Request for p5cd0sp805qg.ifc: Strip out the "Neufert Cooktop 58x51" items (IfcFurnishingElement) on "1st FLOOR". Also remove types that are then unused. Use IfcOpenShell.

First a look at what the model holds.

```python
import ifcopenshell
import ifcopenshell.util.element

model = ifcopenshell.open("p5cd0sp805qg.ifc")
print(model.schema)
storey = next(s for s in model.by_type("IfcBuildingStorey") if s.Name == "1st FLOOR")
furniture = [e for e in ifcopenshell.util.element.get_decomposition(storey) if e.is_a("IfcFurnishingElement")]
seen = {}
for e in furniture:
    element_type = ifcopenshell.util.element.get_type(e)
    name = element_type.Name if element_type not in (None, e) else None
    seen[name] = seen.get(name, 0) + 1
for name, count in sorted(seen.items(), key=str):
    print(count, "x", name)
```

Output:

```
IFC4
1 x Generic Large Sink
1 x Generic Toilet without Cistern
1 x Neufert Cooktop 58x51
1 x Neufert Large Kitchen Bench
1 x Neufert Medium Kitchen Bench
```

```python
import ifcopenshell
import ifcopenshell.api.root
import ifcopenshell.util.element

model = ifcopenshell.open("p5cd0sp805qg.ifc")

storey = next(s for s in model.by_type("IfcBuildingStorey") if s.Name == "1st FLOOR")
furniture = [e for e in ifcopenshell.util.element.get_decomposition(storey) if e.is_a("IfcFurnishingElement")]
targets = [e for e in furniture if (t := ifcopenshell.util.element.get_type(e)) not in (None, e) and t.Name == "Neufert Cooktop 58x51"]
types = {ifcopenshell.util.element.get_type(e) for e in targets} - {None, *targets}

for e in targets:
    ifcopenshell.api.root.remove_product(model, product=e)
print(len(targets), "removed")

unused = [t for t in types if not ifcopenshell.util.element.get_types(t)]
for t in unused:
    ifcopenshell.api.root.remove_product(model, product=t)
print(len(unused), "unused types removed")

model.write("p5cd0sp805qg_updated.ifc")
```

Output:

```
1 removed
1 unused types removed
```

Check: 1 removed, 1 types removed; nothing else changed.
